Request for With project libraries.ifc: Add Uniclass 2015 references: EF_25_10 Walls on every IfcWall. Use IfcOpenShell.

First a look at what the model holds.

```python
import ifcopenshell

model = ifcopenshell.open("With project libraries.ifc")
print(model.schema)
print("classifications:", [c.Name for c in model.by_type("IfcClassification")])
for ifc_class in ("IfcDoor", "IfcRoof", "IfcStair", "IfcWall", "IfcWindow"):
    print(ifc_class, len(model.by_type(ifc_class)))
```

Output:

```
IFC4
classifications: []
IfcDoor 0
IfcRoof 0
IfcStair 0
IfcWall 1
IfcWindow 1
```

```python
import ifcopenshell
import ifcopenshell.api.classification

model = ifcopenshell.open("With project libraries.ifc")

system = ifcopenshell.api.classification.add_classification(model, classification="Uniclass 2015")

codes = {
    "IfcWall": ("EF_25_10", "Walls"),
}
for ifc_class, (code, name) in codes.items():
    products = model.by_type(ifc_class)
    ifcopenshell.api.classification.add_reference(
        model, products=products, classification=system, identification=code, name=name
    )
    print(code, len(products))

model.write("With project libraries_v2.ifc")
```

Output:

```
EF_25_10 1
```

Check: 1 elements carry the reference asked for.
